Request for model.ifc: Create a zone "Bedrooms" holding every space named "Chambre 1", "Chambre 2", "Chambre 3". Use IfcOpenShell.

First a look at what the model holds.

```python
import ifcopenshell

model = ifcopenshell.open("model.ifc")
print(model.schema)
seen = {}
for space in model.by_type("IfcSpace"):
    seen[space.LongName] = seen.get(space.LongName, 0) + 1
for name, count in sorted(seen.items(), key=str):
    print(count, "x", name)
print("zones:", [z.Name for z in model.by_type("IfcZone")][:20])
```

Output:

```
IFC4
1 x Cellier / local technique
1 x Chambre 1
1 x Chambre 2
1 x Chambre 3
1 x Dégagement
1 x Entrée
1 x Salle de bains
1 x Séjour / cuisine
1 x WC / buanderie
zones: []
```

```python
import ifcopenshell
import ifcopenshell.api.group
import ifcopenshell.api.root

model = ifcopenshell.open("model.ifc")

names = {"Chambre 1", "Chambre 2", "Chambre 3"}
spaces = [s for s in model.by_type("IfcSpace") if s.LongName in names]

zone = ifcopenshell.api.root.create_entity(model, ifc_class="IfcZone", name="Bedrooms")
ifcopenshell.api.group.assign_group(model, products=spaces, group=zone)
print(len(spaces), "spaces in", zone.Name)

model.write("model_edited.ifc")
```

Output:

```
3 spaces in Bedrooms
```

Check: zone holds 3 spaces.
